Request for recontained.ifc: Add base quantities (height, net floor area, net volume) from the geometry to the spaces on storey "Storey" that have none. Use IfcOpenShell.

First a look at what the model holds.

```python
import ifcopenshell
import ifcopenshell.util.element
import ifcopenshell.util.unit

model = ifcopenshell.open("recontained.ifc")
print(model.schema)
for unit_type in ("LENGTHUNIT", "AREAUNIT", "VOLUMEUNIT"):
    print(unit_type, ifcopenshell.util.unit.calculate_unit_scale(model, unit_type))
storey = next(s for s in model.by_type("IfcBuildingStorey") if s.Name == "Storey")
spaces = [e for e in ifcopenshell.util.element.get_decomposition(storey) if e.is_a("IfcSpace")]
for e in sorted(spaces, key=lambda e: e.id()):
    print(e.id(), e.is_a(), e.Name, list(ifcopenshell.util.element.get_psets(e, qtos_only=True)), sep=" | ")
```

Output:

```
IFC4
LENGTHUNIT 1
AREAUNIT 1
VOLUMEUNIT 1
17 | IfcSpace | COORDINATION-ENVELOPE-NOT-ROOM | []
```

```python
import ifcopenshell
import ifcopenshell.api.pset
import ifcopenshell.geom
import ifcopenshell.util.element
import ifcopenshell.util.shape
import ifcopenshell.util.unit

model = ifcopenshell.open("recontained.ifc")
unit_scale = ifcopenshell.util.unit.calculate_unit_scale(model)
area_scale = ifcopenshell.util.unit.calculate_unit_scale(model, "AREAUNIT")
volume_scale = ifcopenshell.util.unit.calculate_unit_scale(model, "VOLUMEUNIT")
settings = ifcopenshell.geom.settings()

storey = next(s for s in model.by_type("IfcBuildingStorey") if s.Name == "Storey")
spaces = [e for e in ifcopenshell.util.element.get_decomposition(storey) if e.is_a("IfcSpace")]

for e in sorted(spaces, key=lambda e: e.id()):
    if ifcopenshell.util.element.get_psets(e, qtos_only=True, should_inherit=False):
        continue
    # Geometry comes back in metres, in the element's own axes.
    shape = ifcopenshell.geom.create_shape(settings, e)
    values = {
        "Height": ifcopenshell.util.shape.get_z(shape.geometry) / unit_scale,
        "NetFloorArea": ifcopenshell.util.shape.get_footprint_area(shape.geometry) / area_scale,
        "NetVolume": ifcopenshell.util.shape.get_volume(shape.geometry) / volume_scale,
    }
    qto = ifcopenshell.api.pset.add_qto(model, product=e, name="Qto_SpaceBaseQuantities")
    ifcopenshell.api.pset.edit_qto(model, qto=qto, properties=values)
    print(e.id(), {k: round(v, 3) for k, v in values.items()})

model.write("recontained-out.ifc")
```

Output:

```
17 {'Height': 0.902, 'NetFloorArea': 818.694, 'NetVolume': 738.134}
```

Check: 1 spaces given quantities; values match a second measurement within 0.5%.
